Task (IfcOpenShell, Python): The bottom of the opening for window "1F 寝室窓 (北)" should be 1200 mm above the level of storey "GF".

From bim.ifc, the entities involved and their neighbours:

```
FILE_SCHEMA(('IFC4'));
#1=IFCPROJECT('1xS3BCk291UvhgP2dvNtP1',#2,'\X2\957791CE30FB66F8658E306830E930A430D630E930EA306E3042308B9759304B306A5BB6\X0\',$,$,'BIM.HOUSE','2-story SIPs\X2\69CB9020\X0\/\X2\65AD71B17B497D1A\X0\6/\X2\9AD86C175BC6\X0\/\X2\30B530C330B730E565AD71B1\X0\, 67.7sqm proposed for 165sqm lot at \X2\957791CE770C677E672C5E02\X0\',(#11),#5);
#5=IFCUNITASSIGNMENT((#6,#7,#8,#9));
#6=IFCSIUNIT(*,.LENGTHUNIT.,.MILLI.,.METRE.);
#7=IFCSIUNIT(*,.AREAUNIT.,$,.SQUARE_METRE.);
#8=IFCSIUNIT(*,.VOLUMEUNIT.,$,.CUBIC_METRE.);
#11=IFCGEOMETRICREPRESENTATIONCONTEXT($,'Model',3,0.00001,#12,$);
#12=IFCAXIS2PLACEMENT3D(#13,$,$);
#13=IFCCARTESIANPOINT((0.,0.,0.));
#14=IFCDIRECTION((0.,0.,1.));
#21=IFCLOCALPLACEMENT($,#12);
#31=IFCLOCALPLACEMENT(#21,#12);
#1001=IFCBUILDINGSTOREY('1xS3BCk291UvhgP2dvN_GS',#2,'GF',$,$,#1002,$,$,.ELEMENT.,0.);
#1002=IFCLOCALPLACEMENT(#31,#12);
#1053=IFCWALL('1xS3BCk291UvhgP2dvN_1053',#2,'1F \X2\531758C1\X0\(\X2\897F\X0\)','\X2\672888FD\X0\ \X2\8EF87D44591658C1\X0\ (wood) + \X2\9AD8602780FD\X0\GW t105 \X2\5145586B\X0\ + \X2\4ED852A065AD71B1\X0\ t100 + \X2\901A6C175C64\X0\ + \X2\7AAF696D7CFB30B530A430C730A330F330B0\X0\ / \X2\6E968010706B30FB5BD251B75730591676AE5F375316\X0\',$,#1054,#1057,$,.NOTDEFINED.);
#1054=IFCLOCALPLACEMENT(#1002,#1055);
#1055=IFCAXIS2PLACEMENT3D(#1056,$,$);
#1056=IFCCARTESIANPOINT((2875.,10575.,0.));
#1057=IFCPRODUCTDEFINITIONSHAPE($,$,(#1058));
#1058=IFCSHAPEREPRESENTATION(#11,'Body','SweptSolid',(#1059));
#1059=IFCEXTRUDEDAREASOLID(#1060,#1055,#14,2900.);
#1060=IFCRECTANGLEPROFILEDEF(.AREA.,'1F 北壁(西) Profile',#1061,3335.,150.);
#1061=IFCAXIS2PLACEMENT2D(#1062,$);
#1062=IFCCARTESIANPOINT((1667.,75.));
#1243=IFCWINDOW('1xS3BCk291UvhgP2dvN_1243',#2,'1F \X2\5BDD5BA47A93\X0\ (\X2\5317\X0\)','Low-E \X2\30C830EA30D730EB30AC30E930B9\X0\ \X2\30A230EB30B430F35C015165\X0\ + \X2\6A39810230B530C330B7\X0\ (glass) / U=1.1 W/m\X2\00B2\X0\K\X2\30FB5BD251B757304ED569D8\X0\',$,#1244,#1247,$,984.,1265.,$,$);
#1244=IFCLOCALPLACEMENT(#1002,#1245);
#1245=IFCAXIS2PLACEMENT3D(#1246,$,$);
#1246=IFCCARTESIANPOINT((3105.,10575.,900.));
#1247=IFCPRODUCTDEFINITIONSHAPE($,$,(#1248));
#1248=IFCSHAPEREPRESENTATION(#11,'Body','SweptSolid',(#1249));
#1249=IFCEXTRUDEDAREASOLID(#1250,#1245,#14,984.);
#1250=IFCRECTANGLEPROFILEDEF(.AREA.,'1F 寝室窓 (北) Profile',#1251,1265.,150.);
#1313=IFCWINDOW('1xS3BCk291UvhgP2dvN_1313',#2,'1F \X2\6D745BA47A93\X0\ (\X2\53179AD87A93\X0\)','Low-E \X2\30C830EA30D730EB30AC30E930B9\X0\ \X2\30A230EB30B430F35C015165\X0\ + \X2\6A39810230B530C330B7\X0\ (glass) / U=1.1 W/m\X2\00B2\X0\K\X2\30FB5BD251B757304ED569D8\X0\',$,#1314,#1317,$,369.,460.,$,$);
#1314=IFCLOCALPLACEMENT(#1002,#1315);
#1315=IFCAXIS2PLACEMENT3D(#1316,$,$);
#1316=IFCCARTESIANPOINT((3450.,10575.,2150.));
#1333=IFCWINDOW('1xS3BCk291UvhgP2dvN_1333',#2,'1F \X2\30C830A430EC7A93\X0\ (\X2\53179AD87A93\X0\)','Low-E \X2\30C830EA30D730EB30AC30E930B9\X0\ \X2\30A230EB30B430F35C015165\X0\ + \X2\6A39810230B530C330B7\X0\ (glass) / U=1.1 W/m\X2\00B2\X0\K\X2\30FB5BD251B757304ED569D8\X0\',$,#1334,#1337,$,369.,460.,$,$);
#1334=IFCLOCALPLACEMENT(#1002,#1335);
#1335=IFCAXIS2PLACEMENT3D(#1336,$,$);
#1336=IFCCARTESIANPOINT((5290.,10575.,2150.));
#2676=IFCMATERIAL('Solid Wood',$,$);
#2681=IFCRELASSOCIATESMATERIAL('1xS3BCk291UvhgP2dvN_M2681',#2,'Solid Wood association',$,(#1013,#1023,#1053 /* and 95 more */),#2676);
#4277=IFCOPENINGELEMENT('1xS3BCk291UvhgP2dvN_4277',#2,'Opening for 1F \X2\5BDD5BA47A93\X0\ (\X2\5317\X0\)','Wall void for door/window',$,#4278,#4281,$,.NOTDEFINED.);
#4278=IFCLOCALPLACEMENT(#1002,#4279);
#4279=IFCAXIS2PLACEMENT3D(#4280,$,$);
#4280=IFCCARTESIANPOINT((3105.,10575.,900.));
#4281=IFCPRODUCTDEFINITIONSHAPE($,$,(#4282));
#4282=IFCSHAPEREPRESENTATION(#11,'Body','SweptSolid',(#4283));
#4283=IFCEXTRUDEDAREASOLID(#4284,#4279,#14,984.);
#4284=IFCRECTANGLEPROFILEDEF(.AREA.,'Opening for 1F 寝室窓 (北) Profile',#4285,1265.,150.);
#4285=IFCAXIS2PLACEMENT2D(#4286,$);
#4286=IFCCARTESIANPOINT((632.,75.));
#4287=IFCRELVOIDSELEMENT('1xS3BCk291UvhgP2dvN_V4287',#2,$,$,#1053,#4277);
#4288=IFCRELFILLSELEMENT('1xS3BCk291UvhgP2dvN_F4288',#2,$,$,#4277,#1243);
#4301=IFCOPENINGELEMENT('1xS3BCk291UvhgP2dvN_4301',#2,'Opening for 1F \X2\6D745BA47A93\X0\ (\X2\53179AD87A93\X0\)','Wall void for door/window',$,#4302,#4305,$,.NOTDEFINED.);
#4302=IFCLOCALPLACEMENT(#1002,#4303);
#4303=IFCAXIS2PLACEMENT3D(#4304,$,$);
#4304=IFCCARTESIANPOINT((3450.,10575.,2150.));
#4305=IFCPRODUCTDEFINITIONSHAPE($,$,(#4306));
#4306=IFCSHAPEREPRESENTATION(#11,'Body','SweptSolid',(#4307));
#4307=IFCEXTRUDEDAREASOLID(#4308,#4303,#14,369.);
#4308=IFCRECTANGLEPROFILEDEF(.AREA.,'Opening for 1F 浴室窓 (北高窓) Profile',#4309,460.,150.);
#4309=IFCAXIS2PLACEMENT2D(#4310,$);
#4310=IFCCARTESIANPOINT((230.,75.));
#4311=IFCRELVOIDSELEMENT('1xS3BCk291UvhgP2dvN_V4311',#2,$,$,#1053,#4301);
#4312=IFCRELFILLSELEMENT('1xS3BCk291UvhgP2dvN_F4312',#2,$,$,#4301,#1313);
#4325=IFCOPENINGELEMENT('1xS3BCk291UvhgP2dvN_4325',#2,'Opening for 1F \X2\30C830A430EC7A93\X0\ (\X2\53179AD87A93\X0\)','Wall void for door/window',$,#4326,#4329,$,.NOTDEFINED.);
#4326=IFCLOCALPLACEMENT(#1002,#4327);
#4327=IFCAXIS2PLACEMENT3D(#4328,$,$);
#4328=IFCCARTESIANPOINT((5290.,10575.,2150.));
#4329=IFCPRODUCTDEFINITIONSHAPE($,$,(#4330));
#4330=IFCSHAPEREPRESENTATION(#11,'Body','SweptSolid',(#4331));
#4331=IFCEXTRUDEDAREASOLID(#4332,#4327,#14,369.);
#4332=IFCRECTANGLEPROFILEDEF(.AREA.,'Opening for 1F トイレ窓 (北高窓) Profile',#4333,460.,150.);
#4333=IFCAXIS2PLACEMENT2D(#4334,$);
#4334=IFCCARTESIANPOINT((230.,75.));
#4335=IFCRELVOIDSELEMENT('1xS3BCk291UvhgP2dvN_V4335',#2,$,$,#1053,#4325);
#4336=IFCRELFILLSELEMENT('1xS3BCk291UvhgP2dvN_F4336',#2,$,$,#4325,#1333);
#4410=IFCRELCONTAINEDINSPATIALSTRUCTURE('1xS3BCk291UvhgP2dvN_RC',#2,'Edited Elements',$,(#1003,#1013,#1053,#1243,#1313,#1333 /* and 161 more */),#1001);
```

```python
import numpy as np
import ifcopenshell
import ifcopenshell.api.geometry
import ifcopenshell.geom
import ifcopenshell.util.element
import ifcopenshell.util.placement
import ifcopenshell.util.shape
import ifcopenshell.util.unit

model = ifcopenshell.open("bim.ifc")
unit_scale = ifcopenshell.util.unit.calculate_unit_scale(model)

window = model.by_id(1243)
opening = window.FillsVoids[0].RelatingOpeningElement
storey = ifcopenshell.util.element.get_container(window, ifc_class="IfcBuildingStorey")
level = ifcopenshell.util.placement.get_local_placement(storey.ObjectPlacement)[2, 3]

# The opening's origin need not be at the sill, so measure its lowest point.
shape = ifcopenshell.geom.create_shape(ifcopenshell.geom.settings(), opening)
bottom = ifcopenshell.util.shape.get_shape_bottom_elevation(shape, shape.geometry) / unit_scale
dz = level + 1.2 / unit_scale - bottom

shift = np.array([0.0, 0.0, dz])
# The window is not placed relative to its opening, so move both.
for product in (opening, window):
    matrix = ifcopenshell.util.placement.get_local_placement(product.ObjectPlacement)
    matrix[:3, 3] += shift
    ifcopenshell.api.geometry.edit_object_placement(model, product=product, matrix=matrix, is_si=False)

print(f"moved by {dz * unit_scale:+.3f} m")

model.write("bim_edited.ifc")
```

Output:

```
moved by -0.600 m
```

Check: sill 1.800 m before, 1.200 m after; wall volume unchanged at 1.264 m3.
